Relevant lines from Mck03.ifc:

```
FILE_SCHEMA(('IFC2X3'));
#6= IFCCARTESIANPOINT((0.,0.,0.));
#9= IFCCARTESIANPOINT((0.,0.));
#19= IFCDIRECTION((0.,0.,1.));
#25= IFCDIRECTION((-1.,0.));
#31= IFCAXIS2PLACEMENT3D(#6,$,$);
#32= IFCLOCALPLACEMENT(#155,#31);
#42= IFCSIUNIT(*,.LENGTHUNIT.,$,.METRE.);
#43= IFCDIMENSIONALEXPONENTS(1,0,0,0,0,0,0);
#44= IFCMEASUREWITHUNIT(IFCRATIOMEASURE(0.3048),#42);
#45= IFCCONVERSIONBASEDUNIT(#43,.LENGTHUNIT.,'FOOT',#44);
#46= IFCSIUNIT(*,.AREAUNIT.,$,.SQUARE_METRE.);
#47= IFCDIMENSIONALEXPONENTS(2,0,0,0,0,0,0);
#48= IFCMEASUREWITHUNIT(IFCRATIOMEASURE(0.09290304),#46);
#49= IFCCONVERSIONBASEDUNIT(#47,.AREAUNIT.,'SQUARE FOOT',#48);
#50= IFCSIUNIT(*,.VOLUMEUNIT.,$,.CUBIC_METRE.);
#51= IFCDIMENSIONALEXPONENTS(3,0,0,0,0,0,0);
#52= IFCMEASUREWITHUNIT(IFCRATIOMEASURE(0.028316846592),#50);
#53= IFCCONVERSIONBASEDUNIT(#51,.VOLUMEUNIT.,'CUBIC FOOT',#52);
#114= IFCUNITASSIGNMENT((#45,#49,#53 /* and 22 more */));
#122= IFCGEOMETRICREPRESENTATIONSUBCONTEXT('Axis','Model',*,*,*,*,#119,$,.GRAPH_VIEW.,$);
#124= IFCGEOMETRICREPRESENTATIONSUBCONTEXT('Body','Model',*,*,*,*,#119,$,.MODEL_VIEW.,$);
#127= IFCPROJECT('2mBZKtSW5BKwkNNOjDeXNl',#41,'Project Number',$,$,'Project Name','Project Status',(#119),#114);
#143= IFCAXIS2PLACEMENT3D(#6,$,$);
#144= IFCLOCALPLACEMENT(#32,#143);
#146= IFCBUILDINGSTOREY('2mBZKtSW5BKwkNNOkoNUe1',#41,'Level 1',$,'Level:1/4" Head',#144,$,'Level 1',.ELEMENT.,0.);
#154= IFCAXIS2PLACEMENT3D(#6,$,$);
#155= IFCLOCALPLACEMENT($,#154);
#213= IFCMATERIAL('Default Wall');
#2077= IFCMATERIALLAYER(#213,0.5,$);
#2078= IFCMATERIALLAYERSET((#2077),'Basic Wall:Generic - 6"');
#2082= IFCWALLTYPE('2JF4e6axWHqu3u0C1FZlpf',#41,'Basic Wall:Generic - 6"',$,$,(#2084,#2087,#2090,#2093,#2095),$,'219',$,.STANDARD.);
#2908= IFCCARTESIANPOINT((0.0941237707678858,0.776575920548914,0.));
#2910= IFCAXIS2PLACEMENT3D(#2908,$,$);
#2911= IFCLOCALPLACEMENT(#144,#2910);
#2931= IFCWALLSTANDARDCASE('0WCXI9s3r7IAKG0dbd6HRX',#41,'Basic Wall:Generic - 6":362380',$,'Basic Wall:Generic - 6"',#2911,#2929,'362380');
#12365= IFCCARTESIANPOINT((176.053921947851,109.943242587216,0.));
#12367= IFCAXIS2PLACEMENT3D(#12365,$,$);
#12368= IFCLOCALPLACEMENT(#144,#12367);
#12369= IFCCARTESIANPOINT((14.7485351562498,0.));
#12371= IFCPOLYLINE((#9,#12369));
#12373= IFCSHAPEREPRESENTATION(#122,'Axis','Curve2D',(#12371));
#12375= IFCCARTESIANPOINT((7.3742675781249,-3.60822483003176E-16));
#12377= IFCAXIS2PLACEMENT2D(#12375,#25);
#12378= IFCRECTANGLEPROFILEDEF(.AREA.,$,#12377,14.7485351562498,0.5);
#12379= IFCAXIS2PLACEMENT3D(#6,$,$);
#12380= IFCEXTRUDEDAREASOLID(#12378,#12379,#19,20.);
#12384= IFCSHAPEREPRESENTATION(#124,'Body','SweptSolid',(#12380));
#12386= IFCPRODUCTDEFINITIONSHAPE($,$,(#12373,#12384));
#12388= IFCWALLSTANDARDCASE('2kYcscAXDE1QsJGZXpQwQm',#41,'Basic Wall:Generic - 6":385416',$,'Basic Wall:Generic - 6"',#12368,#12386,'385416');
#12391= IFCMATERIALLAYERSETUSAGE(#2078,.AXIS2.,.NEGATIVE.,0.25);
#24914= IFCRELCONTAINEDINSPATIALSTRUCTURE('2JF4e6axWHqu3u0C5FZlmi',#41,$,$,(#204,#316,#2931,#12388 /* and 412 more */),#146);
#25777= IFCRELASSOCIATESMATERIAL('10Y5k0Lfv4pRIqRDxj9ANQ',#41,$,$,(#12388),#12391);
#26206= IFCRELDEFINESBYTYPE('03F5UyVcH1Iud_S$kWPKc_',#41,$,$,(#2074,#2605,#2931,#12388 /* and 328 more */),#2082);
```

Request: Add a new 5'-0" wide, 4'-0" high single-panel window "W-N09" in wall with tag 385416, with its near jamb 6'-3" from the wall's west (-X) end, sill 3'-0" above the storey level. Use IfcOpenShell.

```python
import numpy as np
import ifcopenshell
import ifcopenshell.api.feature
import ifcopenshell.api.geometry
import ifcopenshell.api.root
import ifcopenshell.api.spatial
import ifcopenshell.api.type
import ifcopenshell.geom
import ifcopenshell.util.element
import ifcopenshell.util.placement
import ifcopenshell.util.representation
import ifcopenshell.util.shape
import ifcopenshell.util.unit

model = ifcopenshell.open("Mck03.ifc")
unit_scale = ifcopenshell.util.unit.calculate_unit_scale(model)
settings = ifcopenshell.geom.settings()


def volume(element):
    """Net volume in cubic metres, openings subtracted."""
    shape = ifcopenshell.geom.create_shape(settings, element)
    return ifcopenshell.util.shape.get_volume(shape.geometry)


wall = model.by_guid("2kYcscAXDE1QsJGZXpQwQm")
storey = ifcopenshell.util.element.get_container(wall, ifc_class="IfcBuildingStorey")
context = ifcopenshell.util.representation.get_context(model, "Model", "Body", "MODEL_VIEW")
before = volume(wall)

width, height, from_end, sill = 1.524, 1.2192, 1.905, 0.9144  # metres

# The wall runs along its own X axis, and the end named is its -X end.
wall_shape = ifcopenshell.geom.create_shape(settings, wall)
x, y, z = ifcopenshell.util.shape.get_vertices(wall_shape.geometry).T
start = x.min() + from_end
face, thickness = float(y.min()), float(y.max() - y.min())
wall_matrix = ifcopenshell.util.placement.get_local_placement(wall.ObjectPlacement)
level = ifcopenshell.util.placement.get_local_placement(storey.ObjectPlacement)[2, 3]


def in_wall(x, y):
    """Placement at x, y metres in the wall's axes, at sill height."""
    matrix = wall_matrix.copy()
    matrix[:, 3] = wall_matrix @ np.array([x / unit_scale, y / unit_scale, 0.0, 1.0])
    matrix[2, 3] = level + sill / unit_scale
    return matrix


# Opening: a box that overshoots both wall faces by 50 mm.
opening = ifcopenshell.api.root.create_entity(model, ifc_class="IfcOpeningElement")
box = ifcopenshell.api.geometry.add_wall_representation(
    model, context=context, length=width, height=height, thickness=thickness + 0.1
)
ifcopenshell.api.geometry.assign_representation(model, product=opening, representation=box)
ifcopenshell.api.geometry.edit_object_placement(model, product=opening, matrix=in_wall(start, face - 0.05), is_si=False)
ifcopenshell.api.feature.add_feature(model, feature=opening, element=wall)

window = ifcopenshell.api.root.create_entity(model, ifc_class="IfcWindow", name="W-N09")
window.OverallWidth, window.OverallHeight = width / unit_scale, height / unit_scale
body = ifcopenshell.api.geometry.add_window_representation(
    model,
    context=context,
    overall_width=window.OverallWidth,
    overall_height=window.OverallHeight,
    partition_type="SINGLE_PANEL",
)
ifcopenshell.api.geometry.assign_representation(model, product=window, representation=body)
ifcopenshell.api.spatial.assign_container(model, products=[window], relating_structure=storey)
fills = ifcopenshell.api.feature.add_filling(model, opening=opening, element=window)
fills.OwnerHistory = window.OwnerHistory  # required in IFC2X3

# IFC2X3 keeps the operation on the window style.
style = ifcopenshell.api.root.create_entity(model, ifc_class="IfcWindowStyle", name="W-N09")
style.OperationType, style.ConstructionType = "SINGLE_PANEL", "NOTDEFINED"
style.ParameterTakesPrecedence = style.Sizeable = False
ifcopenshell.api.type.assign_type(model, related_objects=[window], relating_type=style)

# Centre the window in the wall's thickness.
ifcopenshell.api.geometry.edit_object_placement(model, product=window, matrix=in_wall(start, face), is_si=False)
window_shape = ifcopenshell.geom.create_shape(settings, window)
depth = ifcopenshell.util.shape.get_vertices(window_shape.geometry)[:, 1]
offset = face + thickness / 2 - (depth.min() + depth.max()) / 2
ifcopenshell.api.geometry.edit_object_placement(model, product=window, matrix=in_wall(start, offset), is_si=False)

after = volume(wall)

print(f"wall volume {before:.3f} -> {after:.3f} m3")

model.write("Mck03_edited.ifc")
```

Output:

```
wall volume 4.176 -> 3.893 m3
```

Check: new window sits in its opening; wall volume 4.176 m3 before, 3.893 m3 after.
